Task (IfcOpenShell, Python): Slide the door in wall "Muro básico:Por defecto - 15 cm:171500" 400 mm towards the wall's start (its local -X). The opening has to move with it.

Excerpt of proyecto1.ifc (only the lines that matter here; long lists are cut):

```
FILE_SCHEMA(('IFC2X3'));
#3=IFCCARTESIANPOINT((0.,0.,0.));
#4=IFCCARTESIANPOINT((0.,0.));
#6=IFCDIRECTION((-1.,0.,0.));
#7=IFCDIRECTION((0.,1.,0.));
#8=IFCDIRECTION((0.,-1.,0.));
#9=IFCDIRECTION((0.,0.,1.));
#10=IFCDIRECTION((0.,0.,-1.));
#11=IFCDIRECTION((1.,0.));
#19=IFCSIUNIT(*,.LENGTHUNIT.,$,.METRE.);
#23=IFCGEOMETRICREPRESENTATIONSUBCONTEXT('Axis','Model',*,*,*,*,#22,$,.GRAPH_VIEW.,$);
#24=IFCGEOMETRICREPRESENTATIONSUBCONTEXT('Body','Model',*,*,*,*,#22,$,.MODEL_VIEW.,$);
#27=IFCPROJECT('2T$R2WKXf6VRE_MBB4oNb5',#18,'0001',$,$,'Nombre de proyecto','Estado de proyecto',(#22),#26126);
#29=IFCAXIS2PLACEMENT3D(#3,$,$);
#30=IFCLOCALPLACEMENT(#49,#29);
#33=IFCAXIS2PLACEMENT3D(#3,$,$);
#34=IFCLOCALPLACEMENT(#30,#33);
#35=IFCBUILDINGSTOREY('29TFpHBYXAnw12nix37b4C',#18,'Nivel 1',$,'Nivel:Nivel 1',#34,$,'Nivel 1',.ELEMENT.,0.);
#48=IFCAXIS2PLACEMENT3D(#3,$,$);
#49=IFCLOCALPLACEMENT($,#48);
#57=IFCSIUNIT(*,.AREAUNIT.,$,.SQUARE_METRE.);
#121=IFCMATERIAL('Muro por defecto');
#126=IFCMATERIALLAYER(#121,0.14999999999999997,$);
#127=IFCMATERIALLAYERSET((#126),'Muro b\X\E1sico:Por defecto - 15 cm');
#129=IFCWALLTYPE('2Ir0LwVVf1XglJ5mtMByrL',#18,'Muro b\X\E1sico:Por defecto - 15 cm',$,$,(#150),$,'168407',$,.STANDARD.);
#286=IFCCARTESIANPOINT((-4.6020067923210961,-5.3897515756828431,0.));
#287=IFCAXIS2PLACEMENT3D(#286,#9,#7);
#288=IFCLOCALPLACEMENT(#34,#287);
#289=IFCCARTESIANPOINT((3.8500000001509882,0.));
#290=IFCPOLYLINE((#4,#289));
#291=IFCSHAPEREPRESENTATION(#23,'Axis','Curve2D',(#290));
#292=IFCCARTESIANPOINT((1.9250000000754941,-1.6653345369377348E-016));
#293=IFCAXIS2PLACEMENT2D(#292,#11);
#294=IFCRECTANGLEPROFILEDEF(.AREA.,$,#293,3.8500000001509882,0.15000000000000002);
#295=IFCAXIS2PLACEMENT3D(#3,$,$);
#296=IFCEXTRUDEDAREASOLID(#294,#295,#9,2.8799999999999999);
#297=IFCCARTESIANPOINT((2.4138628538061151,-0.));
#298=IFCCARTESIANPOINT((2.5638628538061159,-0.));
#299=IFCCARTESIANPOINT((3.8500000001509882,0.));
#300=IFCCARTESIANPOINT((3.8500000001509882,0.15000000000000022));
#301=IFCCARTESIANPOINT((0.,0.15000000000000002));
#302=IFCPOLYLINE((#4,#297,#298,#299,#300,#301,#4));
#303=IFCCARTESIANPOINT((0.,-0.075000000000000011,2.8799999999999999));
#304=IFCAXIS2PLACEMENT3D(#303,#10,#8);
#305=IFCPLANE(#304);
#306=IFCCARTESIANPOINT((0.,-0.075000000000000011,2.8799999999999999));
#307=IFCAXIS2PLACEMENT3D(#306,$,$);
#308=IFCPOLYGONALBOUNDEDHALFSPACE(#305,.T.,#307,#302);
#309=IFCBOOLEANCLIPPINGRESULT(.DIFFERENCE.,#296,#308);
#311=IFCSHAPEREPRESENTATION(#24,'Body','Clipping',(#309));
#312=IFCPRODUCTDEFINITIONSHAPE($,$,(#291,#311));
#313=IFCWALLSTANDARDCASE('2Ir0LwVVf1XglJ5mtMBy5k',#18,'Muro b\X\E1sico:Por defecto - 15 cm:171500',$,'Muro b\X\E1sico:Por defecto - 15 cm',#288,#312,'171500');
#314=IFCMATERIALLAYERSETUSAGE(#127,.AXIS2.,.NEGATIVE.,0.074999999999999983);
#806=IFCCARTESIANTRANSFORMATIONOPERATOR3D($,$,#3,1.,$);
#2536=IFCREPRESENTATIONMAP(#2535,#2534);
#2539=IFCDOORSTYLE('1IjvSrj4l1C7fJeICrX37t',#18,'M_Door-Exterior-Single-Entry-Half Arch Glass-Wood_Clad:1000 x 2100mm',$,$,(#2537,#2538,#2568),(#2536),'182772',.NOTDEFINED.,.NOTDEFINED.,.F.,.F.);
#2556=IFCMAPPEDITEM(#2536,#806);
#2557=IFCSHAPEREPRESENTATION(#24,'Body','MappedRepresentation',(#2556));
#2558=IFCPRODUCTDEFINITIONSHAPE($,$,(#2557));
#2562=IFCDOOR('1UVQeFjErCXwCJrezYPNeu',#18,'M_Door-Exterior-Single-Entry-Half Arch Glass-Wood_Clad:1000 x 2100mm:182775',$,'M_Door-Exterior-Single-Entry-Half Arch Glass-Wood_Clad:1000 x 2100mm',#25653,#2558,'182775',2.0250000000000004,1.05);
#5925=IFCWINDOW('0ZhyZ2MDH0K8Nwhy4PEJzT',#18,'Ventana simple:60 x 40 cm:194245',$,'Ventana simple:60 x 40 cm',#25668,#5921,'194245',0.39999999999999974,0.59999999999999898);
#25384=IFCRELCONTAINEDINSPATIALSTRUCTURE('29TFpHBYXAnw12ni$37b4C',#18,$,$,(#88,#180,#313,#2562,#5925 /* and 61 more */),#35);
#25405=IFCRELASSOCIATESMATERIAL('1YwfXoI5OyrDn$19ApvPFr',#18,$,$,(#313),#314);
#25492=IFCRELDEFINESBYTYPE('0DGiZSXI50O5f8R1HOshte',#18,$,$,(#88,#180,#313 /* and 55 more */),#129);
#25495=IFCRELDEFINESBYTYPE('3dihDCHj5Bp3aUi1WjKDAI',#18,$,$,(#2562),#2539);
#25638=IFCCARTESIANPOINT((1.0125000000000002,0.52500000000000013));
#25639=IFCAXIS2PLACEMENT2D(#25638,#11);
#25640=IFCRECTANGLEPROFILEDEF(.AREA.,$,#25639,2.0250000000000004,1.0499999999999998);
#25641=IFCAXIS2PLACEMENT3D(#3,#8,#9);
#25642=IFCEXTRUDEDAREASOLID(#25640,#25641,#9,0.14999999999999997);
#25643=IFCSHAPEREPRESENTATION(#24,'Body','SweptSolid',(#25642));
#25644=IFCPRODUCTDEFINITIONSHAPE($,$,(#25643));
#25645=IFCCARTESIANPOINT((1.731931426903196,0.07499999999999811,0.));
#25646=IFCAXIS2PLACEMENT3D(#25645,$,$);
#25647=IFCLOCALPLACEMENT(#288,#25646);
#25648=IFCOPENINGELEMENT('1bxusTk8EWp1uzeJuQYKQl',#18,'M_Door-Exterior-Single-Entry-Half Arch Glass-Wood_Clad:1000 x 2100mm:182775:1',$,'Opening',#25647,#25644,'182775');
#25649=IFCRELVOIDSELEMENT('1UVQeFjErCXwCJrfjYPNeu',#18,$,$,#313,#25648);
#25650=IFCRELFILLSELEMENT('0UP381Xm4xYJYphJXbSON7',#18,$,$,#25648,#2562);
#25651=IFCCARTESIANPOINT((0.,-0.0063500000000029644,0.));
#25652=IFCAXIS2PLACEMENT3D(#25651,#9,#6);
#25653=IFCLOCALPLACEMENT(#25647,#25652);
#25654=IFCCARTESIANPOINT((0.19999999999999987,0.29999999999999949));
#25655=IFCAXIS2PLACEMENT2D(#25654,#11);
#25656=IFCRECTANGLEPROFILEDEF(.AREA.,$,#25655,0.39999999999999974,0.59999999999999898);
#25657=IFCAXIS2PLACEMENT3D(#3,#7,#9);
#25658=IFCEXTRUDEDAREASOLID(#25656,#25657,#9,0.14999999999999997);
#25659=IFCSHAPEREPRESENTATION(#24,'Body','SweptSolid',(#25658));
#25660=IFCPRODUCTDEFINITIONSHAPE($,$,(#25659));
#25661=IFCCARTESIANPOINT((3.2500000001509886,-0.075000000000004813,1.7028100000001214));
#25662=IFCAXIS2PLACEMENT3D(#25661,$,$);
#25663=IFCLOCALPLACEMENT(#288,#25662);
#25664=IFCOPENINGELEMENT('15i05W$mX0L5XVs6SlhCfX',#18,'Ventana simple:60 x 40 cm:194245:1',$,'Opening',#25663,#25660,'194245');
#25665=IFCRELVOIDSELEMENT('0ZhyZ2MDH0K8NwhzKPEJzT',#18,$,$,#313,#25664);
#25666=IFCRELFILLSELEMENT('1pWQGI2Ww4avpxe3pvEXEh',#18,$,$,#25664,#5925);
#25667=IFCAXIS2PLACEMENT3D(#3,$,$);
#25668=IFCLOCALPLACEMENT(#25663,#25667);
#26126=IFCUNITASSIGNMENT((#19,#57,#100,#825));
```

```python
import ifcopenshell
import ifcopenshell.api.geometry
import ifcopenshell.util.placement

model = ifcopenshell.open("proyecto1.ifc")

door = model.by_id(2562)
opening = door.FillsVoids[0].RelatingOpeningElement
wall = opening.VoidsElements[0].RelatingBuildingElement

wall_matrix = ifcopenshell.util.placement.get_local_placement(wall.ObjectPlacement)
shift = wall_matrix[:3, 0] * -0.4
before = ifcopenshell.util.placement.get_local_placement(door.ObjectPlacement)[:3, 3].copy()

# The door is placed relative to its opening, so it follows when the opening moves.
matrix = ifcopenshell.util.placement.get_local_placement(opening.ObjectPlacement)
matrix[:3, 3] += shift
ifcopenshell.api.geometry.edit_object_placement(
    model, product=opening, matrix=matrix, is_si=False, should_transform_children=True
)

after = ifcopenshell.util.placement.get_local_placement(door.ObjectPlacement)[:3, 3]
print("door moved by", (after - before).round(3) + 0.0)

model.write("proyecto1_rev.ifc")
```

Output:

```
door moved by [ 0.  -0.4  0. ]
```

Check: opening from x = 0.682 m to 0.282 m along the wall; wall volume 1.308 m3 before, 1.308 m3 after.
